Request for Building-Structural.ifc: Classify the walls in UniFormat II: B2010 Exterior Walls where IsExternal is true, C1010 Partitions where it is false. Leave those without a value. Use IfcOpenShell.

First a look at what the model holds.

```python
import ifcopenshell
import ifcopenshell.util.element

model = ifcopenshell.open("Building-Structural.ifc")
print(model.schema)
print("classifications:", [c.Name for c in model.by_type("IfcClassification")])
values = [ifcopenshell.util.element.get_pset(e, "Pset_WallCommon", "IsExternal") for e in model.by_type("IfcWall")]
for value in (True, False, None):
    print("IsExternal", value, values.count(value))
```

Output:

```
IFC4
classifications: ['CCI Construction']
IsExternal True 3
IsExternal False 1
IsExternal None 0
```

```python
import ifcopenshell
import ifcopenshell.api.classification
import ifcopenshell.util.element

model = ifcopenshell.open("Building-Structural.ifc")

system = ifcopenshell.api.classification.add_classification(model, classification="UniFormat II")

walls = model.by_type("IfcWall")
external = {e: ifcopenshell.util.element.get_pset(e, "Pset_WallCommon", "IsExternal") for e in walls}
for flag, code, name in ((True, "B2010", "Exterior Walls"), (False, "C1010", "Partitions")):
    products = [e for e in walls if external[e] is flag]
    ifcopenshell.api.classification.add_reference(
        model, products=products, classification=system, identification=code, name=name
    )
    print(code, len(products))

model.write("Building-Structural-out.ifc")
```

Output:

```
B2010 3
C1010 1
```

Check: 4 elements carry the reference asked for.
